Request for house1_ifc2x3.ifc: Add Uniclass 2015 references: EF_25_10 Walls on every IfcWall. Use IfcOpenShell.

First a look at what the model holds.

```python
import ifcopenshell

model = ifcopenshell.open("house1_ifc2x3.ifc")
print(model.schema)
print("classifications:", [c.Name for c in model.by_type("IfcClassification")])
for ifc_class in ("IfcDoor", "IfcRoof", "IfcStair", "IfcWall", "IfcWindow"):
    print(ifc_class, len(model.by_type(ifc_class)))
```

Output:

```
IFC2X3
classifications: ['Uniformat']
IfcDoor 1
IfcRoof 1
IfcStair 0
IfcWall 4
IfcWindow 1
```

```python
import ifcopenshell
import ifcopenshell.api.classification

model = ifcopenshell.open("house1_ifc2x3.ifc")

# IFC2X3 requires Source and Edition and has no link from the project to the system.
system = model.create_entity("IfcClassification", Source="NBS", Edition="2015", Name="Uniclass 2015")

codes = {
    "IfcWall": ("EF_25_10", "Walls"),
}
for ifc_class, (code, name) in codes.items():
    products = model.by_type(ifc_class)
    ifcopenshell.api.classification.add_reference(
        model, products=products, classification=system, identification=code, name=name
    )
    print(code, len(products))

model.write("house1_ifc2x3_v2.ifc")
```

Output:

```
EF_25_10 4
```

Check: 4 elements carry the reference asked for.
